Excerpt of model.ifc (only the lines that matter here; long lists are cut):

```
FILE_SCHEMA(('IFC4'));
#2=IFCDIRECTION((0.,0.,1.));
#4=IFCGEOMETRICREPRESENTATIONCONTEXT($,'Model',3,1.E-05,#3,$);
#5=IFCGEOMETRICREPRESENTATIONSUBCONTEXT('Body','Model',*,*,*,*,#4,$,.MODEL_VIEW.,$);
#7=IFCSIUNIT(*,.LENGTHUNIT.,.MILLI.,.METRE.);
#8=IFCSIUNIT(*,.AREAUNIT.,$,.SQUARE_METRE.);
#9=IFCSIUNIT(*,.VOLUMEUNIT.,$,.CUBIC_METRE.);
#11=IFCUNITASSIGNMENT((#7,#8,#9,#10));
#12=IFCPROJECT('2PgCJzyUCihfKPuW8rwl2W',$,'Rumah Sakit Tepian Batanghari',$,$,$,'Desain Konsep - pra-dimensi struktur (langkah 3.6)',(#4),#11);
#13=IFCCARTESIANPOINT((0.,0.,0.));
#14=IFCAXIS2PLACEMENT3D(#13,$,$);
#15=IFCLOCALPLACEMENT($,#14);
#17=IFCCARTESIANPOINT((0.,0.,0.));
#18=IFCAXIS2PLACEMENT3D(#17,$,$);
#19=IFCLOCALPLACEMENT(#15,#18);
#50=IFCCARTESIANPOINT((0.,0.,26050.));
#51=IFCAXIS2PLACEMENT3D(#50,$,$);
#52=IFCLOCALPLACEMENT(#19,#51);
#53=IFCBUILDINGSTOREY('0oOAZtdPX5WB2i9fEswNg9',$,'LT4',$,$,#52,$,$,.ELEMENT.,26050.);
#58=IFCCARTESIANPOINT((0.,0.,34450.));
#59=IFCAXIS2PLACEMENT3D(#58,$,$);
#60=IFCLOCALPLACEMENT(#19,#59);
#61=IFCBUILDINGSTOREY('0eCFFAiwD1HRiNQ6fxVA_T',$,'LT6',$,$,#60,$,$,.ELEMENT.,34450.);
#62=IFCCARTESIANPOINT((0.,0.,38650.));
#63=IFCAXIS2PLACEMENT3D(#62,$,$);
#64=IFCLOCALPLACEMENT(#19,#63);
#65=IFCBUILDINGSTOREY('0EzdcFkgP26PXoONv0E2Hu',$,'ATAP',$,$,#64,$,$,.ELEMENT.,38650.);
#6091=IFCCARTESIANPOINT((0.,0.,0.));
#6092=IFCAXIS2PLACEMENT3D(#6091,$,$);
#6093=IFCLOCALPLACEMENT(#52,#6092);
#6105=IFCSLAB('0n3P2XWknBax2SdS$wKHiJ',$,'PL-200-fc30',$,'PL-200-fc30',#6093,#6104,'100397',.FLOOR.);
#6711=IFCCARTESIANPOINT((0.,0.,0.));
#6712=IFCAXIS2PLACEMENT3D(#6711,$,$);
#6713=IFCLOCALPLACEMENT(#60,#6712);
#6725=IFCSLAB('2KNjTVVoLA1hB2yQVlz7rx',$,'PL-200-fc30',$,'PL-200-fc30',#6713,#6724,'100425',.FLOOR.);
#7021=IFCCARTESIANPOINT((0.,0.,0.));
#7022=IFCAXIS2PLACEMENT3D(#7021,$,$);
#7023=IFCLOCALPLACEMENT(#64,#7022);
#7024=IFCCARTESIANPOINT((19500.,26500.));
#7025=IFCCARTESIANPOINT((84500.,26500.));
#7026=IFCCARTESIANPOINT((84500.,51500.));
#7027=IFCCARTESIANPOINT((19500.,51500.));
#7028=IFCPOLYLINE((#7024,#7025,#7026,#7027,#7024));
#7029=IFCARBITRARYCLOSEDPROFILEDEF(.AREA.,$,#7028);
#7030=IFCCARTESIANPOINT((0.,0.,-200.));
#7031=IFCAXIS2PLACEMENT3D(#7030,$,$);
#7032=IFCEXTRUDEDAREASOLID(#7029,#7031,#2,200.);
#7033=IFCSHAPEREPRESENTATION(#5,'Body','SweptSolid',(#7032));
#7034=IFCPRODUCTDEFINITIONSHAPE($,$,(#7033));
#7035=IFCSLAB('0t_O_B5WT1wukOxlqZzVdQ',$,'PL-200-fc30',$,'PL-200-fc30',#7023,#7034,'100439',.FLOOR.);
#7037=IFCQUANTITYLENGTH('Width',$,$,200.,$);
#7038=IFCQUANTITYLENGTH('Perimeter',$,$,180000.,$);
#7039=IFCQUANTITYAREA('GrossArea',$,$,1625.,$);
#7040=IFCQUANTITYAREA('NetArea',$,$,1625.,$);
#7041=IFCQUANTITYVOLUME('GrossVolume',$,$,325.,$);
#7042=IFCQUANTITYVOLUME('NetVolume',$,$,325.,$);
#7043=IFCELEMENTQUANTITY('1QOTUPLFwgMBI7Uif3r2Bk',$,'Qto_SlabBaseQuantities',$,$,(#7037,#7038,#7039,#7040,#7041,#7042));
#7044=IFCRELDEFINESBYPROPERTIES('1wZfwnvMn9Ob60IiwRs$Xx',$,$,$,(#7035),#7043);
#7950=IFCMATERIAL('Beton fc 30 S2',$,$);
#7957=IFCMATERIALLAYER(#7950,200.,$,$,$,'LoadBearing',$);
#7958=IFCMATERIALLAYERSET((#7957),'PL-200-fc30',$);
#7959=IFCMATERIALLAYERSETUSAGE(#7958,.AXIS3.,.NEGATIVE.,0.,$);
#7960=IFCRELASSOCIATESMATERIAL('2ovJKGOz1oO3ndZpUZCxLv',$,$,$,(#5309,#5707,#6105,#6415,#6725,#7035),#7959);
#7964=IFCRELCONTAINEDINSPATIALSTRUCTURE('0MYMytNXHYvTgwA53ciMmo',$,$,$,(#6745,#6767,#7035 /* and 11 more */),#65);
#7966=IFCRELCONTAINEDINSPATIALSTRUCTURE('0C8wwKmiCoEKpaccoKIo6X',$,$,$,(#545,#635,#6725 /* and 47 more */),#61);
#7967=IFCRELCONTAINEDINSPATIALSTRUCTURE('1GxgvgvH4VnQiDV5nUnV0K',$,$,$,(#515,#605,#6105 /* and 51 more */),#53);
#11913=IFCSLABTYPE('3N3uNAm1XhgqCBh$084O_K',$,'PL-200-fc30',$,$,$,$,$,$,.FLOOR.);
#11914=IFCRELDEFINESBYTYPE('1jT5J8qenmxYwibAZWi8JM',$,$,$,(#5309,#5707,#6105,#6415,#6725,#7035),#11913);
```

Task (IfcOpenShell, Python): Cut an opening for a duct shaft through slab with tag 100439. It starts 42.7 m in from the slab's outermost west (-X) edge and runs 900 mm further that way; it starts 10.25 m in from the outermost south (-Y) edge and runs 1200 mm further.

```python
import numpy as np
import ifcopenshell
import ifcopenshell.api.feature
import ifcopenshell.api.geometry
import ifcopenshell.api.pset
import ifcopenshell.api.root
import ifcopenshell.geom
import ifcopenshell.util.element
import ifcopenshell.util.placement
import ifcopenshell.util.representation
import ifcopenshell.util.shape
import ifcopenshell.util.unit

model = ifcopenshell.open("model.ifc")
unit_scale = ifcopenshell.util.unit.calculate_unit_scale(model)
area_scale = ifcopenshell.util.unit.calculate_unit_scale(model, "AREAUNIT")
volume_scale = ifcopenshell.util.unit.calculate_unit_scale(model, "VOLUMEUNIT")
settings = ifcopenshell.geom.settings()


def volume(element):
    """Net volume in cubic metres, openings subtracted."""
    shape = ifcopenshell.geom.create_shape(settings, element)
    return ifcopenshell.util.shape.get_volume(shape.geometry)


slab = model.by_guid("0t_O_B5WT1wukOxlqZzVdQ")
before = volume(slab)

# Extent in the slab's own axes, in metres. The edges named are its -X and -Y sides.
slab_shape = ifcopenshell.geom.create_shape(settings, slab)
vertices = ifcopenshell.util.shape.get_vertices(slab_shape.geometry)
x_min, y_min, bottom = vertices.min(axis=0)
top = vertices[:, 2].max()

opening = ifcopenshell.api.root.create_entity(model, ifc_class="IfcOpeningElement", name="Duct shaft opening", predefined_type="OPENING")
context = ifcopenshell.util.representation.get_context(model, "Model", "Body", "MODEL_VIEW")
width, depth = 0.9, 1.2
outline = [(0.0, 0.0), (width, 0.0), (width, depth), (0.0, depth), (0.0, 0.0)]
# Overshoot both faces by 50 mm so the cut is clean.
shape = ifcopenshell.api.geometry.add_slab_representation(
    model, context=context, depth=top - bottom + 0.1, polyline=outline
)
ifcopenshell.api.geometry.assign_representation(model, product=opening, representation=shape)

matrix = ifcopenshell.util.placement.get_local_placement(slab.ObjectPlacement)
matrix[:, 3] = matrix @ np.append(np.array([x_min + 42.7, y_min + 10.25, bottom - 0.05]) / unit_scale, 1.0)
ifcopenshell.api.geometry.edit_object_placement(model, product=opening, matrix=matrix, is_si=False)
ifcopenshell.api.feature.add_feature(model, feature=opening, element=slab)

after = volume(slab)

# Update the slab's stored quantities.
qto = model.by_id(ifcopenshell.util.element.get_pset(slab, "Qto_SlabBaseQuantities", should_inherit=False)["id"])
ifcopenshell.api.pset.edit_qto(model, qto=qto, properties={
    "NetArea": after / (top - bottom) / area_scale,
    "NetVolume": after / volume_scale,
})

print(f"slab volume {before:.3f} -> {after:.3f} m3")

model.write("model_updated.ifc")
```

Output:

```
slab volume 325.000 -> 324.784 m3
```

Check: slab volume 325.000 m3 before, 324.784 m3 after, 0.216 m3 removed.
